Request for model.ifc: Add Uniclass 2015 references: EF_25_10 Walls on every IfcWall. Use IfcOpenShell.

First a look at what the model holds.

```python
import ifcopenshell

model = ifcopenshell.open("model.ifc")
print(model.schema)
print("classifications:", [c.Name for c in model.by_type("IfcClassification")])
for ifc_class in ("IfcDoor", "IfcRoof", "IfcStair", "IfcWall", "IfcWindow"):
    print(ifc_class, len(model.by_type(ifc_class)))
```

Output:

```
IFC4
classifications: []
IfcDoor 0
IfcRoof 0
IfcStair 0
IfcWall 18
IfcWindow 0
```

```python
import ifcopenshell
import ifcopenshell.api.classification

model = ifcopenshell.open("model.ifc")

system = ifcopenshell.api.classification.add_classification(model, classification="Uniclass 2015")

codes = {
    "IfcWall": ("EF_25_10", "Walls"),
}
for ifc_class, (code, name) in codes.items():
    products = model.by_type(ifc_class)
    ifcopenshell.api.classification.add_reference(
        model, products=products, classification=system, identification=code, name=name
    )
    print(code, len(products))

model.write("model-out.ifc")
```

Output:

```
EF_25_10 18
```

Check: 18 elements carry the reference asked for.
